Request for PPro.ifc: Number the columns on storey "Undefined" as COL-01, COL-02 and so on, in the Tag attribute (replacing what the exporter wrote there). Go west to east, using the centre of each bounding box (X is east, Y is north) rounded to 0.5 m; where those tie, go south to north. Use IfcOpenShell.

First a look at what the model holds.

```python
import ifcopenshell
import ifcopenshell.util.element
import ifcopenshell.util.placement

model = ifcopenshell.open("PPro.ifc")
print(model.schema)
storey = next(s for s in model.by_type("IfcBuildingStorey") if s.Name == "Undefined")
columns = [e for e in ifcopenshell.util.element.get_decomposition(storey) if e.is_a("IfcColumn")]
for e in sorted(columns, key=lambda e: e.id()):
    origin = ifcopenshell.util.placement.get_local_placement(e.ObjectPlacement)[:3, 3]
    print(e.id(), e.Tag, e.Name, origin.round(2) + 0.0, sep=" | ")
```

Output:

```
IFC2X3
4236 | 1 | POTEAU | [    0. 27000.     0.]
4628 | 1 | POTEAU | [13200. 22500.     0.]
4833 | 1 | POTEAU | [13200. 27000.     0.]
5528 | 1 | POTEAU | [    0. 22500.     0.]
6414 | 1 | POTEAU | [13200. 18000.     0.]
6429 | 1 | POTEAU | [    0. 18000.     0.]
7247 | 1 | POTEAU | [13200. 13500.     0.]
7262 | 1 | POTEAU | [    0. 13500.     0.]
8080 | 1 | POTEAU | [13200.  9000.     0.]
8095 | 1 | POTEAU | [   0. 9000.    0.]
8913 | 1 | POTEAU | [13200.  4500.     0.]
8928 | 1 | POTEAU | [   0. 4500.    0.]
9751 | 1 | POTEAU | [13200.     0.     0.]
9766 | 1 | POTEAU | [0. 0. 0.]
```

```python
import ifcopenshell
import ifcopenshell.geom
import ifcopenshell.util.element
import ifcopenshell.util.shape

model = ifcopenshell.open("PPro.ifc")
settings = ifcopenshell.geom.settings()
settings.set("use-world-coords", True)


def centre(element):
    shape = ifcopenshell.geom.create_shape(settings, element)
    return ifcopenshell.util.shape.get_bbox_centroid(shape.geometry)


storey = next(s for s in model.by_type("IfcBuildingStorey") if s.Name == "Undefined")
columns = [e for e in ifcopenshell.util.element.get_decomposition(storey) if e.is_a("IfcColumn")]

# Insertion points can sit at a corner or the storey origin, so sort by the geometry (in metres).
centres = {e: centre(e) for e in columns}
columns.sort(key=lambda e: (round(centres[e][0] / 0.5), centres[e][1]))

for i, e in enumerate(columns, start=1):
    number = f"COL-{i:02d}"
    e.Tag = number
    print(e.id(), number)

model.write("PPro-out.ifc")
```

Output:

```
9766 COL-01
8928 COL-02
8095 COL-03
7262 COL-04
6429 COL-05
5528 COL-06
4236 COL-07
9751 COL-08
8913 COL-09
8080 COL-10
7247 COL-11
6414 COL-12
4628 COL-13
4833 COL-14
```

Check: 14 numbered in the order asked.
